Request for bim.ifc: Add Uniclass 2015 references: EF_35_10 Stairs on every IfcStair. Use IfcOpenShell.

First a look at what the model holds.

```python
import ifcopenshell

model = ifcopenshell.open("bim.ifc")
print(model.schema)
print("classifications:", [c.Name for c in model.by_type("IfcClassification")])
for ifc_class in ("IfcDoor", "IfcRoof", "IfcStair", "IfcWall", "IfcWindow"):
    print(ifc_class, len(model.by_type(ifc_class)))
```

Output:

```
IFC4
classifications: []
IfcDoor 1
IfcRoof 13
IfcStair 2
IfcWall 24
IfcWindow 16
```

```python
import ifcopenshell
import ifcopenshell.api.classification

model = ifcopenshell.open("bim.ifc")

system = ifcopenshell.api.classification.add_classification(model, classification="Uniclass 2015")

codes = {
    "IfcStair": ("EF_35_10", "Stairs"),
}
for ifc_class, (code, name) in codes.items():
    products = model.by_type(ifc_class)
    ifcopenshell.api.classification.add_reference(
        model, products=products, classification=system, identification=code, name=name
    )
    print(code, len(products))

model.write("bim_updated.ifc")
```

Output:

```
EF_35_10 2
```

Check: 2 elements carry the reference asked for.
